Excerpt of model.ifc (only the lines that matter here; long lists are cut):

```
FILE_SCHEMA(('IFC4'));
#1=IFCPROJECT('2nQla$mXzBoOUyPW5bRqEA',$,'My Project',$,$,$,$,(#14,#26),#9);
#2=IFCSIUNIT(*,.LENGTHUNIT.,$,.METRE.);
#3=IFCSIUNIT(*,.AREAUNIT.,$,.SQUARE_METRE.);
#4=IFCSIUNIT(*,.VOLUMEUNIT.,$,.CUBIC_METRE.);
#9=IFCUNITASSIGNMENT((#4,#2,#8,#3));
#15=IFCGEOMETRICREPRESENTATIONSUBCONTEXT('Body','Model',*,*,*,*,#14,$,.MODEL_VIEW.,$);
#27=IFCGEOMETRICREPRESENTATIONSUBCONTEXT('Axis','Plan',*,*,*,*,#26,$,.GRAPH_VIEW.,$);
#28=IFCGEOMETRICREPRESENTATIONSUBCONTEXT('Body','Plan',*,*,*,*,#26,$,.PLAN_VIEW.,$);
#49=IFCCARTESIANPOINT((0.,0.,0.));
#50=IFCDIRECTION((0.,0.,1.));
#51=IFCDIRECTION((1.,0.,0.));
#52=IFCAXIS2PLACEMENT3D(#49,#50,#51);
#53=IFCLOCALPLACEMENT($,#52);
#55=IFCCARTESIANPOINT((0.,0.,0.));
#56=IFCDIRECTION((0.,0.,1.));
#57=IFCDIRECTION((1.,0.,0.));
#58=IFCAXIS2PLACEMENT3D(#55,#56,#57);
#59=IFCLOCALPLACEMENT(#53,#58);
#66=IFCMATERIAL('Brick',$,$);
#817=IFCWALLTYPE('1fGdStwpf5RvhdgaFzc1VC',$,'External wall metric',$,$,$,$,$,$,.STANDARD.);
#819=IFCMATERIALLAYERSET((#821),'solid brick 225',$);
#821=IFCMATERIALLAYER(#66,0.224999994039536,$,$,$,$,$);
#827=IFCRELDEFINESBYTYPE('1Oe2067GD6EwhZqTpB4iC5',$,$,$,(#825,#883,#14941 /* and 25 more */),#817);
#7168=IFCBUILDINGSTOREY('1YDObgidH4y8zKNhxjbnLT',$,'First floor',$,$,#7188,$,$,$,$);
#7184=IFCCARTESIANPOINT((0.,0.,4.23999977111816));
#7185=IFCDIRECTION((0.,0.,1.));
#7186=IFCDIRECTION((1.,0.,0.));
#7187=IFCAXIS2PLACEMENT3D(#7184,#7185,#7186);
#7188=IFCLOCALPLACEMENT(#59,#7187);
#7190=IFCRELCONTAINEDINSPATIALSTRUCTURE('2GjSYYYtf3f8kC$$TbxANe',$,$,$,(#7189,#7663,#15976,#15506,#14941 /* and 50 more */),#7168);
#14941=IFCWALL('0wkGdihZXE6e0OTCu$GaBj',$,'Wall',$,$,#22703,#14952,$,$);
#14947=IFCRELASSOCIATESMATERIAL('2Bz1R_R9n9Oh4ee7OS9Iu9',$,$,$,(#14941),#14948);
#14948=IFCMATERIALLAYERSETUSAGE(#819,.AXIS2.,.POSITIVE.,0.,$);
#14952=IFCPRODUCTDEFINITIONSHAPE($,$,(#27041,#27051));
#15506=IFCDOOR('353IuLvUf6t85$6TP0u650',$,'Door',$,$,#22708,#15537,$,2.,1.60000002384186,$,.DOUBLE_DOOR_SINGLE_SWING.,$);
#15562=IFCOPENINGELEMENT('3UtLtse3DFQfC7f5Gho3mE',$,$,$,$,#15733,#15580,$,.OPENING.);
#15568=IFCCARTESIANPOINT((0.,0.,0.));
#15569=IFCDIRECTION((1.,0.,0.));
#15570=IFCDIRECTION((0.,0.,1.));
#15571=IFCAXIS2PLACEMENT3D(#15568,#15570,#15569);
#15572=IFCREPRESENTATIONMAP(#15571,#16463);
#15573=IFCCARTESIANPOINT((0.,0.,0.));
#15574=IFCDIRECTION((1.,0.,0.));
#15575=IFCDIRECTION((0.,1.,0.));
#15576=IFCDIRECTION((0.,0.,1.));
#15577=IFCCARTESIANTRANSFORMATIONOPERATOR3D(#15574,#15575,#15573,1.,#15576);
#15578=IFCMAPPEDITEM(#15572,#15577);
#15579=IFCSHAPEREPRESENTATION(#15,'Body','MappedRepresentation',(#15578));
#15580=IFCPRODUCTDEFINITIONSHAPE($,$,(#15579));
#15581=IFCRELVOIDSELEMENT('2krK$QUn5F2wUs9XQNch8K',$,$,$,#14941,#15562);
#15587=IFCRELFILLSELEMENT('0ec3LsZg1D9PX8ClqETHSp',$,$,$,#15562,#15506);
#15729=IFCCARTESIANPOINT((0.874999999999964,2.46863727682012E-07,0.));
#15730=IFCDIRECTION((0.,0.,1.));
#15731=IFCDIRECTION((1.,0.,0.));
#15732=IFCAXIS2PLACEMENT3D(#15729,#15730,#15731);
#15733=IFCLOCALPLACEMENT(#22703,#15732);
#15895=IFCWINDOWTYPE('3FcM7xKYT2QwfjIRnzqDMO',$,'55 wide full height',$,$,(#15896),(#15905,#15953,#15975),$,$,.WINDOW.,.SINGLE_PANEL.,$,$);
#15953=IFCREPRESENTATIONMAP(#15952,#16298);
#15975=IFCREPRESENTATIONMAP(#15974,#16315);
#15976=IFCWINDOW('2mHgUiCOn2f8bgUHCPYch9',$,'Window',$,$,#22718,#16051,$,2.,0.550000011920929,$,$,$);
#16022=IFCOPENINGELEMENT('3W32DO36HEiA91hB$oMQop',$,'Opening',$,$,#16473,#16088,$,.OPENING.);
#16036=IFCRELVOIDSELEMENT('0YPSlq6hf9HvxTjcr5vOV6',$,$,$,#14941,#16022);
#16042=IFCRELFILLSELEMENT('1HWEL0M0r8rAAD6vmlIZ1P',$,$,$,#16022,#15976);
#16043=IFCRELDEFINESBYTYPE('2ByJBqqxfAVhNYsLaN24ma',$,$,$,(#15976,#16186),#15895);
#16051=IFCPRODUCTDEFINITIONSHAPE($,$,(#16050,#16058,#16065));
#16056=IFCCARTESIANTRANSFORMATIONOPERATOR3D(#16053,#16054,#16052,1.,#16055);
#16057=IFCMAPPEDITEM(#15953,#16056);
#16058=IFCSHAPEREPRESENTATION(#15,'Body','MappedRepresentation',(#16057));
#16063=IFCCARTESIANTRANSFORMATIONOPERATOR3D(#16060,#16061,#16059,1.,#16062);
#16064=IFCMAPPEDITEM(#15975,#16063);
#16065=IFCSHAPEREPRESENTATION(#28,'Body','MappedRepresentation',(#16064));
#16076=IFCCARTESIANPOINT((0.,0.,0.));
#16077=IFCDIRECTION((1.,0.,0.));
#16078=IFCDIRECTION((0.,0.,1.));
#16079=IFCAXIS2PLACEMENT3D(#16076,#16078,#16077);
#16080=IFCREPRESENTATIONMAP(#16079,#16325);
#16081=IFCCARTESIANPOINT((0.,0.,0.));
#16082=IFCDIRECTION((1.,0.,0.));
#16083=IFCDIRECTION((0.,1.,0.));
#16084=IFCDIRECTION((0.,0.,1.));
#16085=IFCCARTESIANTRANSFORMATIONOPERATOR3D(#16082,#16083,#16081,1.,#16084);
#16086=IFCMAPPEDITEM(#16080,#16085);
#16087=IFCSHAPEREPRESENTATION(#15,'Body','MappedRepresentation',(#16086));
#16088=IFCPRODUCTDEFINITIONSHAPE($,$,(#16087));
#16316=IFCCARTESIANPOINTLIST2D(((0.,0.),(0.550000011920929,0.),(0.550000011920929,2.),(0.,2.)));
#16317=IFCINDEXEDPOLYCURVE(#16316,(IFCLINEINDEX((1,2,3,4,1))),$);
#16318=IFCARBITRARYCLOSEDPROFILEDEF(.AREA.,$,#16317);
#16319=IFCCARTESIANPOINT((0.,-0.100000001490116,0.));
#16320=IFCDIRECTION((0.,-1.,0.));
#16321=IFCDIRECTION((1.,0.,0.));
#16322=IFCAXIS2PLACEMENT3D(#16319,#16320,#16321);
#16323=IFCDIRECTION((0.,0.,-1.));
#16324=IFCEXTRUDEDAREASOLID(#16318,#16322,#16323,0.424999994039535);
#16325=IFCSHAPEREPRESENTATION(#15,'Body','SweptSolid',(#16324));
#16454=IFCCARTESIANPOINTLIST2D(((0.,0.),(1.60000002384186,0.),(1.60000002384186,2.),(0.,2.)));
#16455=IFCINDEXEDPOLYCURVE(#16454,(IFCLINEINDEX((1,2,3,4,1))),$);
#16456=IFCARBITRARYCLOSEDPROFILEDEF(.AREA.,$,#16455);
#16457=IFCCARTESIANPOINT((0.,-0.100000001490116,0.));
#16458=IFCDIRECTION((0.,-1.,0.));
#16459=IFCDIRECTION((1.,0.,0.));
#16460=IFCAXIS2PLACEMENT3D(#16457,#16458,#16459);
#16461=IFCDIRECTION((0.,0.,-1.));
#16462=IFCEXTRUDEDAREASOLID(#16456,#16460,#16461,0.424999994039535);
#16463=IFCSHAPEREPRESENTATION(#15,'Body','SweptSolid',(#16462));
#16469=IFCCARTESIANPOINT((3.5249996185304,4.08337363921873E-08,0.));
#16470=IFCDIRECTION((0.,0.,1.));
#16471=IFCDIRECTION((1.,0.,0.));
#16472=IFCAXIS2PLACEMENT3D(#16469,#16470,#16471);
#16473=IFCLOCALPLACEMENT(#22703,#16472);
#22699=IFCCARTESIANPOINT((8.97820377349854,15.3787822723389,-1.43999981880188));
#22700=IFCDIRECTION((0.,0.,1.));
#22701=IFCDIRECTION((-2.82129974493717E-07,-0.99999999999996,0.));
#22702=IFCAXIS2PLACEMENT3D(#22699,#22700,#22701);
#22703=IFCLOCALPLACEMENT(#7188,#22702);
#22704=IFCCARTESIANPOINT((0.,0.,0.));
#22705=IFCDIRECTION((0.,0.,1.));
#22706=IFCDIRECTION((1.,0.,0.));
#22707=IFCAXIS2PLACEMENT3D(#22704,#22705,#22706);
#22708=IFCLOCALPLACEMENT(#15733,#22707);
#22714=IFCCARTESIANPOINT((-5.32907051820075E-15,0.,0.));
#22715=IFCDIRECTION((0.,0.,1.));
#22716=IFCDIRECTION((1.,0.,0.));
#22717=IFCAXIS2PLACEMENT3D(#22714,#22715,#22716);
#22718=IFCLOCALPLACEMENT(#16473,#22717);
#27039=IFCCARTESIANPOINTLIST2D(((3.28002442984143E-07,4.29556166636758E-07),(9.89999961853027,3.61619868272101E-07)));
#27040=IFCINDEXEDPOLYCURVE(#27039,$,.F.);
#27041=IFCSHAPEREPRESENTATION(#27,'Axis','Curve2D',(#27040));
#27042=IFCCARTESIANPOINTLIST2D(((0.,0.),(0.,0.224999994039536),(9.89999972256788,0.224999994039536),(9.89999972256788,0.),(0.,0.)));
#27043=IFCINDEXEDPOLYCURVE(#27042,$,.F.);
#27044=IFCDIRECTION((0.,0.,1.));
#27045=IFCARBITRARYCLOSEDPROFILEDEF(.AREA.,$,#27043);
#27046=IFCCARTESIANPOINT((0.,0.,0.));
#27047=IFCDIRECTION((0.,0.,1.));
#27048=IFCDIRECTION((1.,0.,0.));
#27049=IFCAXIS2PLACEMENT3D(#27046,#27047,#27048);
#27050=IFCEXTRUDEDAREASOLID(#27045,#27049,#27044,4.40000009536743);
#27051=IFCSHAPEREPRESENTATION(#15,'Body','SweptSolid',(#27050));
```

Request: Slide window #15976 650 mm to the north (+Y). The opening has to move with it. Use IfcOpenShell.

```python
import ifcopenshell
import ifcopenshell.api.geometry
import ifcopenshell.util.placement
import ifcopenshell.util.unit

model = ifcopenshell.open("model.ifc")
unit_scale = ifcopenshell.util.unit.calculate_unit_scale(model)

window = model.by_guid("2mHgUiCOn2f8bgUHCPYch9")
opening = window.FillsVoids[0].RelatingOpeningElement
wall = opening.VoidsElements[0].RelatingBuildingElement

wall_matrix = ifcopenshell.util.placement.get_local_placement(wall.ObjectPlacement)
shift = wall_matrix[:3, 0] * -0.65 / unit_scale
before = ifcopenshell.util.placement.get_local_placement(window.ObjectPlacement)[:3, 3].copy()

# The window is placed relative to its opening, so it follows when the opening moves.
matrix = ifcopenshell.util.placement.get_local_placement(opening.ObjectPlacement)
matrix[:3, 3] += shift
ifcopenshell.api.geometry.edit_object_placement(
    model, product=opening, matrix=matrix, is_si=False, should_transform_children=True
)

after = ifcopenshell.util.placement.get_local_placement(window.ObjectPlacement)[:3, 3]
print("window moved by", (after - before).round(3) + 0.0)

model.write("model_edited.ifc")
```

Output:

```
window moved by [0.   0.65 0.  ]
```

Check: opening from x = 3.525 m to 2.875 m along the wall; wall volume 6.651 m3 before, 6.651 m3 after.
